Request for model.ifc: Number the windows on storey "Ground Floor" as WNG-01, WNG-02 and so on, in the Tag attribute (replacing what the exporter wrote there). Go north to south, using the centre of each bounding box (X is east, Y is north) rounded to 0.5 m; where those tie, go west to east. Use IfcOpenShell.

First a look at what the model holds.

```python
import ifcopenshell
import ifcopenshell.util.element
import ifcopenshell.util.placement

model = ifcopenshell.open("model.ifc")
print(model.schema)
storey = next(s for s in model.by_type("IfcBuildingStorey") if s.Name == "Ground Floor")
windows = [e for e in ifcopenshell.util.element.get_decomposition(storey) if e.is_a("IfcWindow")]
for e in sorted(windows, key=lambda e: e.id()):
    origin = ifcopenshell.util.placement.get_local_placement(e.ObjectPlacement)[:3, 3]
    print(e.id(), e.Tag, e.Name, origin.round(2) + 0.0, sep=" | ")
```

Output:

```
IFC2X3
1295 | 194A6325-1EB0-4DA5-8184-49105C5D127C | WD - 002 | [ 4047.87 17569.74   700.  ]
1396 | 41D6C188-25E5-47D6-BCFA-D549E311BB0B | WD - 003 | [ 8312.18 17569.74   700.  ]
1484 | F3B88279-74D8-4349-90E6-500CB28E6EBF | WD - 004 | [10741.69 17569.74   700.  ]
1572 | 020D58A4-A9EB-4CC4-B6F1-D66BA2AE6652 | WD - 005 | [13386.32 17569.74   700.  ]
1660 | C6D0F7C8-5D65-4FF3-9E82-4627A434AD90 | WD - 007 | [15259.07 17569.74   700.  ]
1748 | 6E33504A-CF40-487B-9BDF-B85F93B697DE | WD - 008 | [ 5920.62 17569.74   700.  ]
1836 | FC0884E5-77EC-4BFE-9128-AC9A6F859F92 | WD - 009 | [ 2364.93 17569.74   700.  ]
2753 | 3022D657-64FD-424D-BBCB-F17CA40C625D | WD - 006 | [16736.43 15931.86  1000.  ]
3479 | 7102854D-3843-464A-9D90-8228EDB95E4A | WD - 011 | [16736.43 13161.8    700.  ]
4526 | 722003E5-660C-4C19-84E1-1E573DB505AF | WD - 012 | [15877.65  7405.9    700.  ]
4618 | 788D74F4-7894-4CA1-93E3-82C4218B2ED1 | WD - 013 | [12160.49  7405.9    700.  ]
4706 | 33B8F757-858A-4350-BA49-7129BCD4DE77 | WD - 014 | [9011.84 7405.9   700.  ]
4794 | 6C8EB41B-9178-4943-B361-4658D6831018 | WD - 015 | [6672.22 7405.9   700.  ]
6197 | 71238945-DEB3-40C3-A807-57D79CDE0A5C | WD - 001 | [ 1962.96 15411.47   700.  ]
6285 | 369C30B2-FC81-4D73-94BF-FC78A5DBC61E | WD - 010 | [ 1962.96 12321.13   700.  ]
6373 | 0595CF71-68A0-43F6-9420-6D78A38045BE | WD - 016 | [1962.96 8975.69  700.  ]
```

```python
import ifcopenshell
import ifcopenshell.geom
import ifcopenshell.util.element
import ifcopenshell.util.shape

model = ifcopenshell.open("model.ifc")
settings = ifcopenshell.geom.settings()
settings.set("use-world-coords", True)


def centre(element):
    shape = ifcopenshell.geom.create_shape(settings, element)
    return ifcopenshell.util.shape.get_bbox_centroid(shape.geometry)


storey = next(s for s in model.by_type("IfcBuildingStorey") if s.Name == "Ground Floor")
windows = [e for e in ifcopenshell.util.element.get_decomposition(storey) if e.is_a("IfcWindow")]

# Insertion points can sit at a corner or the storey origin, so sort by the geometry (in metres).
centres = {e: centre(e) for e in windows}
windows.sort(key=lambda e: (-round(centres[e][1] / 0.5), centres[e][0]))

for i, e in enumerate(windows, start=1):
    number = f"WNG-{i:02d}"
    e.Tag = number
    print(e.id(), number)

model.write("model_v2.ifc")
```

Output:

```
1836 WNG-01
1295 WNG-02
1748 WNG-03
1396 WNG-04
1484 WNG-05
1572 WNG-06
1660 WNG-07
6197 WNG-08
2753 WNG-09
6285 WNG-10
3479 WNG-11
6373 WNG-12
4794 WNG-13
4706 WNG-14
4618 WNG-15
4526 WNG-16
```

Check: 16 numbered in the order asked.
